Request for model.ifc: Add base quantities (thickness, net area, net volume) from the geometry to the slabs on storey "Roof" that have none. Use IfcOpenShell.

First a look at what the model holds.

```python
import ifcopenshell
import ifcopenshell.util.element
import ifcopenshell.util.unit

model = ifcopenshell.open("model.ifc")
print(model.schema)
for unit_type in ("LENGTHUNIT", "AREAUNIT", "VOLUMEUNIT"):
    print(unit_type, ifcopenshell.util.unit.calculate_unit_scale(model, unit_type))
storey = next(s for s in model.by_type("IfcBuildingStorey") if s.Name == "Roof")
slabs = [e for e in ifcopenshell.util.element.get_decomposition(storey) if e.is_a("IfcSlab")]
for e in sorted(slabs, key=lambda e: e.id()):
    print(e.id(), e.is_a(), e.Name, list(ifcopenshell.util.element.get_psets(e, qtos_only=True)), sep=" | ")
```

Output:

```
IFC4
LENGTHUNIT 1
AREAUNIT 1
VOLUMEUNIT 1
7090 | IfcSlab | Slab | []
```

```python
import ifcopenshell
import ifcopenshell.api.pset
import ifcopenshell.geom
import ifcopenshell.util.element
import ifcopenshell.util.shape
import ifcopenshell.util.unit

model = ifcopenshell.open("model.ifc")
unit_scale = ifcopenshell.util.unit.calculate_unit_scale(model)
area_scale = ifcopenshell.util.unit.calculate_unit_scale(model, "AREAUNIT")
volume_scale = ifcopenshell.util.unit.calculate_unit_scale(model, "VOLUMEUNIT")
settings = ifcopenshell.geom.settings()

storey = next(s for s in model.by_type("IfcBuildingStorey") if s.Name == "Roof")
slabs = [e for e in ifcopenshell.util.element.get_decomposition(storey) if e.is_a("IfcSlab")]

for e in sorted(slabs, key=lambda e: e.id()):
    if ifcopenshell.util.element.get_psets(e, qtos_only=True, should_inherit=False):
        continue
    # Geometry comes back in metres, in the element's own axes.
    shape = ifcopenshell.geom.create_shape(settings, e)
    values = {
        "Width": ifcopenshell.util.shape.get_z(shape.geometry) / unit_scale,
        "NetArea": ifcopenshell.util.shape.get_footprint_area(shape.geometry) / area_scale,
        "NetVolume": ifcopenshell.util.shape.get_volume(shape.geometry) / volume_scale,
    }
    qto = ifcopenshell.api.pset.add_qto(model, product=e, name="Qto_SlabBaseQuantities")
    ifcopenshell.api.pset.edit_qto(model, qto=qto, properties=values)
    print(e.id(), {k: round(v, 3) for k, v in values.items()})

model.write("model_v2.ifc")
```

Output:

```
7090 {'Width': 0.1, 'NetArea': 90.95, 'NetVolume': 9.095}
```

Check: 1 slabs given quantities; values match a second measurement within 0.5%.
